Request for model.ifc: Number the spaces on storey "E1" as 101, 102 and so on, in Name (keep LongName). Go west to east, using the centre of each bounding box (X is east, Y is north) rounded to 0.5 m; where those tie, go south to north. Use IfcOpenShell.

First a look at what the model holds.

```python
import ifcopenshell
import ifcopenshell.util.element
import ifcopenshell.util.placement

model = ifcopenshell.open("model.ifc")
print(model.schema)
storey = next(s for s in model.by_type("IfcBuildingStorey") if s.Name == "E1")
spaces = [e for e in ifcopenshell.util.element.get_decomposition(storey) if e.is_a("IfcSpace")]
for e in sorted(spaces, key=lambda e: e.id()):
    origin = ifcopenshell.util.placement.get_local_placement(e.ObjectPlacement)[:3, 3]
    print(e.id(), e.Name, e.LongName, origin.round(2) + 0.0, sep=" | ")
```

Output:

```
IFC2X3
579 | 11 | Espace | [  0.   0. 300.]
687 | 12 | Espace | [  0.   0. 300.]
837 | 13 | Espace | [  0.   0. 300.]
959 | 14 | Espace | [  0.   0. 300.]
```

```python
import ifcopenshell
import ifcopenshell.geom
import ifcopenshell.util.element
import ifcopenshell.util.shape

model = ifcopenshell.open("model.ifc")
settings = ifcopenshell.geom.settings()
settings.set("use-world-coords", True)


def centre(element):
    shape = ifcopenshell.geom.create_shape(settings, element)
    return ifcopenshell.util.shape.get_bbox_centroid(shape.geometry)


storey = next(s for s in model.by_type("IfcBuildingStorey") if s.Name == "E1")
spaces = [e for e in ifcopenshell.util.element.get_decomposition(storey) if e.is_a("IfcSpace")]

# Insertion points can sit at a corner or the storey origin, so sort by the geometry (in metres).
centres = {e: centre(e) for e in spaces}
spaces.sort(key=lambda e: (round(centres[e][0] / 0.5), centres[e][1]))

for i, e in enumerate(spaces, start=1):
    number = f"1{i:02d}"
    e.Name = number
    print(e.id(), number)

model.write("model_edited.ifc")
```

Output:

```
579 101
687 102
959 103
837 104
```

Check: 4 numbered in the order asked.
